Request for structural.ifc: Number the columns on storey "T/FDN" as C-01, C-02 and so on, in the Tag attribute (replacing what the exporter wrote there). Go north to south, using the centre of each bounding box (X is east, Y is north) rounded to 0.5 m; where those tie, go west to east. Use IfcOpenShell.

First a look at what the model holds.

```python
import ifcopenshell
import ifcopenshell.util.element
import ifcopenshell.util.placement

model = ifcopenshell.open("structural.ifc")
print(model.schema)
storey = next(s for s in model.by_type("IfcBuildingStorey") if s.Name == "T/FDN")
columns = [e for e in ifcopenshell.util.element.get_decomposition(storey) if e.is_a("IfcColumn")]
for e in sorted(columns, key=lambda e: e.id()):
    origin = ifcopenshell.util.placement.get_local_placement(e.ObjectPlacement)[:3, 3]
    print(e.id(), e.Tag, e.Name, origin.round(2) + 0.0, sep=" | ")
```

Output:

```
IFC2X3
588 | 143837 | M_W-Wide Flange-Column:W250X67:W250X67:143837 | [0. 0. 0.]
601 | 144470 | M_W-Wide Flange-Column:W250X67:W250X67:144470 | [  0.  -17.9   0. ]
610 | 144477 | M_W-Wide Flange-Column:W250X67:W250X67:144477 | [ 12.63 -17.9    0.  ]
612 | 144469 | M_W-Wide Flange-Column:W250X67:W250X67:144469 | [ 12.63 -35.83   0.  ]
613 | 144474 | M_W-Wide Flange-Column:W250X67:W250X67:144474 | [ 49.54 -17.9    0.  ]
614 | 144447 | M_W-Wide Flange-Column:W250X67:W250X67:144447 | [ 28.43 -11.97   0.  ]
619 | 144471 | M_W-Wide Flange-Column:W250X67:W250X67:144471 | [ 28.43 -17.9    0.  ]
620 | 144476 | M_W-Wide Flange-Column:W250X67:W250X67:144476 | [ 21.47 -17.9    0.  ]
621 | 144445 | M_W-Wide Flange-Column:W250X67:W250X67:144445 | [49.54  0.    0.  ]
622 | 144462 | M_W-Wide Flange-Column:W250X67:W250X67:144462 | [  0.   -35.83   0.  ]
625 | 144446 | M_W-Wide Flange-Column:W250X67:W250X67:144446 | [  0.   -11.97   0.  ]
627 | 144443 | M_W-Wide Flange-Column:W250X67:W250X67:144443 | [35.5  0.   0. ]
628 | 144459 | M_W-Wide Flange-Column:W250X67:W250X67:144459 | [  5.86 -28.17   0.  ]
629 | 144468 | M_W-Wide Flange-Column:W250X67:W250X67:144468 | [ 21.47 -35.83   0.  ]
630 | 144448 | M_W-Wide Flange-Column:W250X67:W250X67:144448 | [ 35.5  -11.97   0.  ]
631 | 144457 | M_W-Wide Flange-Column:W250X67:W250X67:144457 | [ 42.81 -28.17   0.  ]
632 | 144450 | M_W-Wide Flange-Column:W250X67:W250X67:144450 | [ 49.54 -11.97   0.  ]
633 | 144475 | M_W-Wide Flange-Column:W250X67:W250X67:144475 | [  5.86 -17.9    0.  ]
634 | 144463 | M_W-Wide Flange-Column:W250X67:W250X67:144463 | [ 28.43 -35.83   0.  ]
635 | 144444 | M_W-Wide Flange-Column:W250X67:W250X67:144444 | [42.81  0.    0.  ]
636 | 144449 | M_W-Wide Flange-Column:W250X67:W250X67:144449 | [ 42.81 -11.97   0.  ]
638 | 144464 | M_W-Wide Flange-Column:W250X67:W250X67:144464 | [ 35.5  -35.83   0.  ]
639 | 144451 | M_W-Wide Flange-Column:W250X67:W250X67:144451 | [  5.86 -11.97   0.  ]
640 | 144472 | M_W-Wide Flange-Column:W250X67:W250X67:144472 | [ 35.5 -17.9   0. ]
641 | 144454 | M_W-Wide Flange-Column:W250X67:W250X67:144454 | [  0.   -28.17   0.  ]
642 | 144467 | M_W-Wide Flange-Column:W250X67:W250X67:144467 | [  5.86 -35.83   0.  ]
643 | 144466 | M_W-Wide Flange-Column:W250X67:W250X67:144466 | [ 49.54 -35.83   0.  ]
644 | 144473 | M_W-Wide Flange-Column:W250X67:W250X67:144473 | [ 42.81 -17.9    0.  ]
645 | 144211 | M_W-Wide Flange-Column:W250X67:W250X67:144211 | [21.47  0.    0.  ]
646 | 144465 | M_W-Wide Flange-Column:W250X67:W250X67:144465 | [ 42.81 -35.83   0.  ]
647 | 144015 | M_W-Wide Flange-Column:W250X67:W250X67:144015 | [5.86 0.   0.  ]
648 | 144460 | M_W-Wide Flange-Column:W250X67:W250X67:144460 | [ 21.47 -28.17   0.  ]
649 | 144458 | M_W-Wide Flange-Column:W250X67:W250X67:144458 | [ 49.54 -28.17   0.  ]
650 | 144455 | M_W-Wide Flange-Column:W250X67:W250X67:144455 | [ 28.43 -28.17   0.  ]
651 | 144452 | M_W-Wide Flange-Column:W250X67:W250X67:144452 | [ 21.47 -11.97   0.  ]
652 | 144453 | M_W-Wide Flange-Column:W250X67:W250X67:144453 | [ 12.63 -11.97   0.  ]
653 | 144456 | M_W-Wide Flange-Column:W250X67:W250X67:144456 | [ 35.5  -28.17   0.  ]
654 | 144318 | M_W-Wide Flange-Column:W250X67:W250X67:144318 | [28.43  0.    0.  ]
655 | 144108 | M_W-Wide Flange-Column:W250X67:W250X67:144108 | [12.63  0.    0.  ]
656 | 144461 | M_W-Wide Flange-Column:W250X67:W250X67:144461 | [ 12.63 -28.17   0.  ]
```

```python
import ifcopenshell
import ifcopenshell.geom
import ifcopenshell.util.element
import ifcopenshell.util.shape

model = ifcopenshell.open("structural.ifc")
settings = ifcopenshell.geom.settings()
settings.set("use-world-coords", True)


def centre(element):
    shape = ifcopenshell.geom.create_shape(settings, element)
    return ifcopenshell.util.shape.get_bbox_centroid(shape.geometry)


storey = next(s for s in model.by_type("IfcBuildingStorey") if s.Name == "T/FDN")
columns = [e for e in ifcopenshell.util.element.get_decomposition(storey) if e.is_a("IfcColumn")]

# Insertion points can sit at a corner or the storey origin, so sort by the geometry (in metres).
centres = {e: centre(e) for e in columns}
columns.sort(key=lambda e: (-round(centres[e][1] / 0.5), centres[e][0]))

for i, e in enumerate(columns, start=1):
    number = f"C-{i:02d}"
    e.Tag = number
    print(e.id(), number)

model.write("structural_edited.ifc")
```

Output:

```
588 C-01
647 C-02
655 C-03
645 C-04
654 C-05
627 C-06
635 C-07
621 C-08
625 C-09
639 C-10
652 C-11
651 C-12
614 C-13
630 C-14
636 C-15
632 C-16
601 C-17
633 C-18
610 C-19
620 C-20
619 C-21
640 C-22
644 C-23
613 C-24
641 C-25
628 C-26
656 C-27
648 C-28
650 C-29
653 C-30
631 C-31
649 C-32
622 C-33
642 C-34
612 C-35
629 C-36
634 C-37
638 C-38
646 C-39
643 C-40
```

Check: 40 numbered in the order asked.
